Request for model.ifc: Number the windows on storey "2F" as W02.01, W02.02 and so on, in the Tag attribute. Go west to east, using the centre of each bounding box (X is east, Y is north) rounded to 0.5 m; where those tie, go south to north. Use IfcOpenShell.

First a look at what the model holds.

```python
import ifcopenshell
import ifcopenshell.util.element
import ifcopenshell.util.placement

model = ifcopenshell.open("model.ifc")
print(model.schema)
storey = next(s for s in model.by_type("IfcBuildingStorey") if s.Name == "2F")
windows = [e for e in ifcopenshell.util.element.get_decomposition(storey) if e.is_a("IfcWindow")]
for e in sorted(windows, key=lambda e: e.id()):
    origin = ifcopenshell.util.placement.get_local_placement(e.ObjectPlacement)[:3, 3]
    print(e.id(), e.Tag, e.Name, origin.round(2) + 0.0, sep=" | ")
```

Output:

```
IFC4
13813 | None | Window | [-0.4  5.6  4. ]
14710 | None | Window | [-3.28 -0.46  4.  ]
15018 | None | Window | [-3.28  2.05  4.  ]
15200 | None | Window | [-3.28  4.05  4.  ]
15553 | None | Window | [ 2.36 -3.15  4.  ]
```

```python
import ifcopenshell
import ifcopenshell.geom
import ifcopenshell.util.element
import ifcopenshell.util.shape

model = ifcopenshell.open("model.ifc")
settings = ifcopenshell.geom.settings()
settings.set("use-world-coords", True)


def centre(element):
    shape = ifcopenshell.geom.create_shape(settings, element)
    return ifcopenshell.util.shape.get_bbox_centroid(shape.geometry)


storey = next(s for s in model.by_type("IfcBuildingStorey") if s.Name == "2F")
windows = [e for e in ifcopenshell.util.element.get_decomposition(storey) if e.is_a("IfcWindow")]

# Insertion points can sit at a corner or the storey origin, so sort by the geometry (in metres).
centres = {e: centre(e) for e in windows}
windows.sort(key=lambda e: (round(centres[e][0] / 0.5), centres[e][1]))

for i, e in enumerate(windows, start=1):
    number = f"W02.{i:02d}"
    e.Tag = number
    print(e.id(), number)

model.write("model_updated.ifc")
```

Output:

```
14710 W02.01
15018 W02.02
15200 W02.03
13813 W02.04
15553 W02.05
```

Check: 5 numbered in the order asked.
